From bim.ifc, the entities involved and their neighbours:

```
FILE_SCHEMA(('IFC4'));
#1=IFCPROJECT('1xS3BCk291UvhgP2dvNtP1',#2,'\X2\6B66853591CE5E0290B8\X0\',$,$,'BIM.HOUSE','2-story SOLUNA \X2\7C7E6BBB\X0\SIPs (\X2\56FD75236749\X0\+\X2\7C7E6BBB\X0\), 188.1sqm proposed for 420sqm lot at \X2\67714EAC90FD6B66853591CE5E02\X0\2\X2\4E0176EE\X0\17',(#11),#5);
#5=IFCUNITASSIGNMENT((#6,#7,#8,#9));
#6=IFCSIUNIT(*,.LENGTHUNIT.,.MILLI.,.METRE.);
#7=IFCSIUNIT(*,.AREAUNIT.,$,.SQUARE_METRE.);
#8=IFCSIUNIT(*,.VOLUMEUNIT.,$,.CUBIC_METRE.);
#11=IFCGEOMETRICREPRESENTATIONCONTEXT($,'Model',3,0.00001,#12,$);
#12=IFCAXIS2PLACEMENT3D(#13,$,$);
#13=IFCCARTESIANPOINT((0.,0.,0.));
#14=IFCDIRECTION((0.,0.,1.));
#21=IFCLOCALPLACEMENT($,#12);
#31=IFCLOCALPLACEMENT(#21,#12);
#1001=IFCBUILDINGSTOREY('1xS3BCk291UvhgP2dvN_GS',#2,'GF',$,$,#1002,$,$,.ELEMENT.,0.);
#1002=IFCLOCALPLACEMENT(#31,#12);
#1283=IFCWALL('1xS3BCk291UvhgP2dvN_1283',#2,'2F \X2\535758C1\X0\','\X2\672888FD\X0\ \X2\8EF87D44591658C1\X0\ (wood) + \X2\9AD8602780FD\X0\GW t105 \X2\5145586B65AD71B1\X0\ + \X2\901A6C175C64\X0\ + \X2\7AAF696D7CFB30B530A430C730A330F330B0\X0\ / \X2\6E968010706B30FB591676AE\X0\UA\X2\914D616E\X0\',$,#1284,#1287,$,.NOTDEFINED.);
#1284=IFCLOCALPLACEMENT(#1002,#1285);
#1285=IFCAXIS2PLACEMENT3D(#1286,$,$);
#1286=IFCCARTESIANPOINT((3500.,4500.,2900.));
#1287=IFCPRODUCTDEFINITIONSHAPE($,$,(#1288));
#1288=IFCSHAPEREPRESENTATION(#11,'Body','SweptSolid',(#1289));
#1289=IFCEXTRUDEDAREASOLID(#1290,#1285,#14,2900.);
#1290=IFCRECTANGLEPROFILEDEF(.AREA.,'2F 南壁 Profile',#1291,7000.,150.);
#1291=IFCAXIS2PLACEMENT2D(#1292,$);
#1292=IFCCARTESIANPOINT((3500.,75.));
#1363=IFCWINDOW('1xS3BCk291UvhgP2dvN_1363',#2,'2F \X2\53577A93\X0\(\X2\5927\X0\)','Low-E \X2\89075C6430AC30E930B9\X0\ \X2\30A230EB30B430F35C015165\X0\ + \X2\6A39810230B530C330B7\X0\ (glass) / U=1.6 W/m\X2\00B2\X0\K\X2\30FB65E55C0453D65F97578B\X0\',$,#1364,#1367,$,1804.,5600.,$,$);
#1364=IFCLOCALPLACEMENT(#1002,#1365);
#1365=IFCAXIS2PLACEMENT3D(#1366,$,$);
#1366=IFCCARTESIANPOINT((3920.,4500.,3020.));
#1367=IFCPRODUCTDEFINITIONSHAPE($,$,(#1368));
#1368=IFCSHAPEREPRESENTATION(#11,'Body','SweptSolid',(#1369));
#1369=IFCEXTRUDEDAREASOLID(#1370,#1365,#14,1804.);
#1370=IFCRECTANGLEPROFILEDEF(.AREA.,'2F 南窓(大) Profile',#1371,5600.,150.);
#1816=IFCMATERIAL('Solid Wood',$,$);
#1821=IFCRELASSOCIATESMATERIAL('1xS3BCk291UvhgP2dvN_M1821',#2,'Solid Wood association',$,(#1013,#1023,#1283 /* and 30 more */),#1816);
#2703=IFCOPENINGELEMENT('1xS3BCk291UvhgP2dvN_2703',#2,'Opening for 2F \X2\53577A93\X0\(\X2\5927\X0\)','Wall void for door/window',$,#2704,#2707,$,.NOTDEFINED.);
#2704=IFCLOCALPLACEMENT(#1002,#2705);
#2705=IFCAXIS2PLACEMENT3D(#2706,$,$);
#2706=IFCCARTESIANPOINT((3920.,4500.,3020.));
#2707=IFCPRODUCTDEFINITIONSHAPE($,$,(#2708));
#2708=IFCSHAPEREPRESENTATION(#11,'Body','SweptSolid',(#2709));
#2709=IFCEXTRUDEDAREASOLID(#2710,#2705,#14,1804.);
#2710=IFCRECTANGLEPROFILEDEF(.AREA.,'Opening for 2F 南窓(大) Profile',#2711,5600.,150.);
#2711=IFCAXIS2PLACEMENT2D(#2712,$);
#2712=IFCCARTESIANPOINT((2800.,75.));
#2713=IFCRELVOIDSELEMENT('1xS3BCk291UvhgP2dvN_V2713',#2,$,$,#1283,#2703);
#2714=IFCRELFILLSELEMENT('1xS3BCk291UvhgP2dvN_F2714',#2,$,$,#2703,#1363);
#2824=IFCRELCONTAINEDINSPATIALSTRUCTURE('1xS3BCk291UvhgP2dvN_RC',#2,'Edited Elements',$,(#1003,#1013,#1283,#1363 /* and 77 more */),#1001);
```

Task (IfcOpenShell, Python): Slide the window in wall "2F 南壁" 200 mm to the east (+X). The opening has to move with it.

```python
import ifcopenshell
import ifcopenshell.api.geometry
import ifcopenshell.util.placement

model = ifcopenshell.open("bim.ifc")

window = model.by_id(1363)
opening = window.FillsVoids[0].RelatingOpeningElement
wall = opening.VoidsElements[0].RelatingBuildingElement

wall_matrix = ifcopenshell.util.placement.get_local_placement(wall.ObjectPlacement)
shift = wall_matrix[:3, 0] * 200.0
before = ifcopenshell.util.placement.get_local_placement(window.ObjectPlacement)[:3, 3].copy()

# The window is not placed relative to its opening, so move both.
for product in (opening, window):
    matrix = ifcopenshell.util.placement.get_local_placement(product.ObjectPlacement)
    matrix[:3, 3] += shift
    ifcopenshell.api.geometry.edit_object_placement(model, product=product, matrix=matrix, is_si=False)

after = ifcopenshell.util.placement.get_local_placement(window.ObjectPlacement)[:3, 3]
print("window moved by", (after - before).round(3) + 0.0)

model.write("bim_v2.ifc")
```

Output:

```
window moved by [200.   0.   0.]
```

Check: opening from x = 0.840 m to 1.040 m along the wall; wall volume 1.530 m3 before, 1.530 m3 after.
